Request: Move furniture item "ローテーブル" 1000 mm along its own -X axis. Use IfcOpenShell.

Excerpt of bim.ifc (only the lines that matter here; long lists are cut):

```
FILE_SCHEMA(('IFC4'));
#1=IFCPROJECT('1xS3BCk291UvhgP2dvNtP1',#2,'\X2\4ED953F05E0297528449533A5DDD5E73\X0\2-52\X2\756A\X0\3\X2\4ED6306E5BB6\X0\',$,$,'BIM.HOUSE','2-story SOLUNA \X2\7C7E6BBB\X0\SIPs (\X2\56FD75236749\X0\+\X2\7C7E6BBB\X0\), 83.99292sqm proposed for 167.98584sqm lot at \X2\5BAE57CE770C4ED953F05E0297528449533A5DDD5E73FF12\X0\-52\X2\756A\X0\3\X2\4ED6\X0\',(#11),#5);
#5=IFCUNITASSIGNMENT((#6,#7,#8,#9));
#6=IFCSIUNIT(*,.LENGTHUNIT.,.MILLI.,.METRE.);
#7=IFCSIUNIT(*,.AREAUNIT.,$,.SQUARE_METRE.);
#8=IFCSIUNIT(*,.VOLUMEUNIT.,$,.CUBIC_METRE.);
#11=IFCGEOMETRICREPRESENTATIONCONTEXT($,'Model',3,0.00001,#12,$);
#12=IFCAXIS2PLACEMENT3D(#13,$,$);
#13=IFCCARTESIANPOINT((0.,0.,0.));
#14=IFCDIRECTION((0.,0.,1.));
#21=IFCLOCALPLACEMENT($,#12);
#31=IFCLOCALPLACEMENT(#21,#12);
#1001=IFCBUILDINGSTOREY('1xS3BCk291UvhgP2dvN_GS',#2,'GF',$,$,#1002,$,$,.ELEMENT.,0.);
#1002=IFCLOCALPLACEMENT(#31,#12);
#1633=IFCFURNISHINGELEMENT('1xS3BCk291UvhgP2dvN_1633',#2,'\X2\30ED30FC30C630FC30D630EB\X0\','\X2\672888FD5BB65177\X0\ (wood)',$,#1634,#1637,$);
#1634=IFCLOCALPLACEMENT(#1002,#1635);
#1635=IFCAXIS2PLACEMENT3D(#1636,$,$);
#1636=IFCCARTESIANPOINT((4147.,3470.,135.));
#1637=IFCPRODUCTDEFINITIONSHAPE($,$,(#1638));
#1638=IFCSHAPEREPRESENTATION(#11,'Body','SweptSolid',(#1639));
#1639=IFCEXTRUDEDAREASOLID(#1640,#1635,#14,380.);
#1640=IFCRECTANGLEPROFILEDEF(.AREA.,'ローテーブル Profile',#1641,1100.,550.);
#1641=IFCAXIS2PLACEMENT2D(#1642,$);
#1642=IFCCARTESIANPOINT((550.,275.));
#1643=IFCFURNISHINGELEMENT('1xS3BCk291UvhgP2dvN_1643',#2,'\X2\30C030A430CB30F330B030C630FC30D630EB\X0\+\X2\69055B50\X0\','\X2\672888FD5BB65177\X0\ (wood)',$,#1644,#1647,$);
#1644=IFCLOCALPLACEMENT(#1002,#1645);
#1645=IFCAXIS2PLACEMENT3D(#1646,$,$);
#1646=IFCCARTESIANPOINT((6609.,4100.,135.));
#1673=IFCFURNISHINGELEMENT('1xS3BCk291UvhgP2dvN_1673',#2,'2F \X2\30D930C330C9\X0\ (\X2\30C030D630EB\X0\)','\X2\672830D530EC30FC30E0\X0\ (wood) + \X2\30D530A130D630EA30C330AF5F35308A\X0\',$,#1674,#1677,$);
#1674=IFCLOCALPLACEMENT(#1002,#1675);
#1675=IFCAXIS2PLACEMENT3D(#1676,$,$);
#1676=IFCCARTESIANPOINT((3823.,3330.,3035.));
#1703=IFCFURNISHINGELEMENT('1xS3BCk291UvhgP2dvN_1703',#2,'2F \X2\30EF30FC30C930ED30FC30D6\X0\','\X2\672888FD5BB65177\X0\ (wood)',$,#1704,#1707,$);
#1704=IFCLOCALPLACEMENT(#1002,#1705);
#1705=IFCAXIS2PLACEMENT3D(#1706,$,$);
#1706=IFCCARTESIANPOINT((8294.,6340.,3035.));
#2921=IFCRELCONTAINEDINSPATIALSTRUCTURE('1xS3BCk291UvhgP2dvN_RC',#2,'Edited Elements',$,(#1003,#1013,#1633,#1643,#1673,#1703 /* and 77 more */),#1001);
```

```python
import ifcopenshell
import ifcopenshell.api.geometry
import ifcopenshell.util.placement
import ifcopenshell.util.unit

model = ifcopenshell.open("bim.ifc")
unit_scale = ifcopenshell.util.unit.calculate_unit_scale(model)

item = model.by_guid("1xS3BCk291UvhgP2dvN_1633")
matrix = ifcopenshell.util.placement.get_local_placement(item.ObjectPlacement)
matrix[:3, 3] -= matrix[:3, 0] * 1 / unit_scale
ifcopenshell.api.geometry.edit_object_placement(model, product=item, matrix=matrix, is_si=False)

print(ifcopenshell.util.placement.get_local_placement(item.ObjectPlacement).round(3) + 0.0)

model.write("bim_edited.ifc")
```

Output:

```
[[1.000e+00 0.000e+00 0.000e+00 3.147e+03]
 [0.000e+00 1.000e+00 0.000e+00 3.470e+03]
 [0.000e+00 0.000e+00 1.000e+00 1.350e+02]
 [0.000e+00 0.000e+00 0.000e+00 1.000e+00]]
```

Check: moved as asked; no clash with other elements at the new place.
